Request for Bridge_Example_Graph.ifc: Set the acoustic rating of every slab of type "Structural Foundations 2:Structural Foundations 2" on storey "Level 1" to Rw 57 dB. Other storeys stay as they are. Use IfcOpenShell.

First a look at what the model holds.

```python
import ifcopenshell
import ifcopenshell.util.element

model = ifcopenshell.open("Bridge_Example_Graph.ifc")
print(model.schema)
storey = next(s for s in model.by_type("IfcBuildingStorey") if s.Name == "Level 1")
slabs = [e for e in ifcopenshell.util.element.get_decomposition(storey) if e.is_a("IfcSlab")]
seen = {}
for e in slabs:
    element_type = ifcopenshell.util.element.get_type(e)
    key = (element_type.Name if element_type != e and element_type else None, ifcopenshell.util.element.get_pset(e, "Pset_SlabCommon", "AcousticRating"))
    seen[key] = seen.get(key, 0) + 1
for (name, value), count in sorted(seen.items(), key=str):
    print(count, "x", name, "|", value)
```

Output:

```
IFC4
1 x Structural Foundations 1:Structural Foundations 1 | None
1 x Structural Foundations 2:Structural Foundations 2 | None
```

```python
import ifcopenshell
import ifcopenshell.api.pset
import ifcopenshell.util.element

model = ifcopenshell.open("Bridge_Example_Graph.ifc")

storey = next(s for s in model.by_type("IfcBuildingStorey") if s.Name == "Level 1")
slabs = [e for e in ifcopenshell.util.element.get_decomposition(storey) if e.is_a("IfcSlab")]

count = 0
for e in slabs:
    element_type = ifcopenshell.util.element.get_type(e)
    if element_type in (None, e) or element_type.Name != "Structural Foundations 2:Structural Foundations 2":
        continue
    # add_pset returns the element's existing set when there is one.
    pset = ifcopenshell.api.pset.add_pset(model, product=e, name="Pset_SlabCommon")
    ifcopenshell.api.pset.edit_pset(model, pset=pset, properties={"AcousticRating": "Rw 57 dB"})
    count += 1

print(count, "slabs updated")

model.write("Bridge_Example_Graph_v2.ifc")
```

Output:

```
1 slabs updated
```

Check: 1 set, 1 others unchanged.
